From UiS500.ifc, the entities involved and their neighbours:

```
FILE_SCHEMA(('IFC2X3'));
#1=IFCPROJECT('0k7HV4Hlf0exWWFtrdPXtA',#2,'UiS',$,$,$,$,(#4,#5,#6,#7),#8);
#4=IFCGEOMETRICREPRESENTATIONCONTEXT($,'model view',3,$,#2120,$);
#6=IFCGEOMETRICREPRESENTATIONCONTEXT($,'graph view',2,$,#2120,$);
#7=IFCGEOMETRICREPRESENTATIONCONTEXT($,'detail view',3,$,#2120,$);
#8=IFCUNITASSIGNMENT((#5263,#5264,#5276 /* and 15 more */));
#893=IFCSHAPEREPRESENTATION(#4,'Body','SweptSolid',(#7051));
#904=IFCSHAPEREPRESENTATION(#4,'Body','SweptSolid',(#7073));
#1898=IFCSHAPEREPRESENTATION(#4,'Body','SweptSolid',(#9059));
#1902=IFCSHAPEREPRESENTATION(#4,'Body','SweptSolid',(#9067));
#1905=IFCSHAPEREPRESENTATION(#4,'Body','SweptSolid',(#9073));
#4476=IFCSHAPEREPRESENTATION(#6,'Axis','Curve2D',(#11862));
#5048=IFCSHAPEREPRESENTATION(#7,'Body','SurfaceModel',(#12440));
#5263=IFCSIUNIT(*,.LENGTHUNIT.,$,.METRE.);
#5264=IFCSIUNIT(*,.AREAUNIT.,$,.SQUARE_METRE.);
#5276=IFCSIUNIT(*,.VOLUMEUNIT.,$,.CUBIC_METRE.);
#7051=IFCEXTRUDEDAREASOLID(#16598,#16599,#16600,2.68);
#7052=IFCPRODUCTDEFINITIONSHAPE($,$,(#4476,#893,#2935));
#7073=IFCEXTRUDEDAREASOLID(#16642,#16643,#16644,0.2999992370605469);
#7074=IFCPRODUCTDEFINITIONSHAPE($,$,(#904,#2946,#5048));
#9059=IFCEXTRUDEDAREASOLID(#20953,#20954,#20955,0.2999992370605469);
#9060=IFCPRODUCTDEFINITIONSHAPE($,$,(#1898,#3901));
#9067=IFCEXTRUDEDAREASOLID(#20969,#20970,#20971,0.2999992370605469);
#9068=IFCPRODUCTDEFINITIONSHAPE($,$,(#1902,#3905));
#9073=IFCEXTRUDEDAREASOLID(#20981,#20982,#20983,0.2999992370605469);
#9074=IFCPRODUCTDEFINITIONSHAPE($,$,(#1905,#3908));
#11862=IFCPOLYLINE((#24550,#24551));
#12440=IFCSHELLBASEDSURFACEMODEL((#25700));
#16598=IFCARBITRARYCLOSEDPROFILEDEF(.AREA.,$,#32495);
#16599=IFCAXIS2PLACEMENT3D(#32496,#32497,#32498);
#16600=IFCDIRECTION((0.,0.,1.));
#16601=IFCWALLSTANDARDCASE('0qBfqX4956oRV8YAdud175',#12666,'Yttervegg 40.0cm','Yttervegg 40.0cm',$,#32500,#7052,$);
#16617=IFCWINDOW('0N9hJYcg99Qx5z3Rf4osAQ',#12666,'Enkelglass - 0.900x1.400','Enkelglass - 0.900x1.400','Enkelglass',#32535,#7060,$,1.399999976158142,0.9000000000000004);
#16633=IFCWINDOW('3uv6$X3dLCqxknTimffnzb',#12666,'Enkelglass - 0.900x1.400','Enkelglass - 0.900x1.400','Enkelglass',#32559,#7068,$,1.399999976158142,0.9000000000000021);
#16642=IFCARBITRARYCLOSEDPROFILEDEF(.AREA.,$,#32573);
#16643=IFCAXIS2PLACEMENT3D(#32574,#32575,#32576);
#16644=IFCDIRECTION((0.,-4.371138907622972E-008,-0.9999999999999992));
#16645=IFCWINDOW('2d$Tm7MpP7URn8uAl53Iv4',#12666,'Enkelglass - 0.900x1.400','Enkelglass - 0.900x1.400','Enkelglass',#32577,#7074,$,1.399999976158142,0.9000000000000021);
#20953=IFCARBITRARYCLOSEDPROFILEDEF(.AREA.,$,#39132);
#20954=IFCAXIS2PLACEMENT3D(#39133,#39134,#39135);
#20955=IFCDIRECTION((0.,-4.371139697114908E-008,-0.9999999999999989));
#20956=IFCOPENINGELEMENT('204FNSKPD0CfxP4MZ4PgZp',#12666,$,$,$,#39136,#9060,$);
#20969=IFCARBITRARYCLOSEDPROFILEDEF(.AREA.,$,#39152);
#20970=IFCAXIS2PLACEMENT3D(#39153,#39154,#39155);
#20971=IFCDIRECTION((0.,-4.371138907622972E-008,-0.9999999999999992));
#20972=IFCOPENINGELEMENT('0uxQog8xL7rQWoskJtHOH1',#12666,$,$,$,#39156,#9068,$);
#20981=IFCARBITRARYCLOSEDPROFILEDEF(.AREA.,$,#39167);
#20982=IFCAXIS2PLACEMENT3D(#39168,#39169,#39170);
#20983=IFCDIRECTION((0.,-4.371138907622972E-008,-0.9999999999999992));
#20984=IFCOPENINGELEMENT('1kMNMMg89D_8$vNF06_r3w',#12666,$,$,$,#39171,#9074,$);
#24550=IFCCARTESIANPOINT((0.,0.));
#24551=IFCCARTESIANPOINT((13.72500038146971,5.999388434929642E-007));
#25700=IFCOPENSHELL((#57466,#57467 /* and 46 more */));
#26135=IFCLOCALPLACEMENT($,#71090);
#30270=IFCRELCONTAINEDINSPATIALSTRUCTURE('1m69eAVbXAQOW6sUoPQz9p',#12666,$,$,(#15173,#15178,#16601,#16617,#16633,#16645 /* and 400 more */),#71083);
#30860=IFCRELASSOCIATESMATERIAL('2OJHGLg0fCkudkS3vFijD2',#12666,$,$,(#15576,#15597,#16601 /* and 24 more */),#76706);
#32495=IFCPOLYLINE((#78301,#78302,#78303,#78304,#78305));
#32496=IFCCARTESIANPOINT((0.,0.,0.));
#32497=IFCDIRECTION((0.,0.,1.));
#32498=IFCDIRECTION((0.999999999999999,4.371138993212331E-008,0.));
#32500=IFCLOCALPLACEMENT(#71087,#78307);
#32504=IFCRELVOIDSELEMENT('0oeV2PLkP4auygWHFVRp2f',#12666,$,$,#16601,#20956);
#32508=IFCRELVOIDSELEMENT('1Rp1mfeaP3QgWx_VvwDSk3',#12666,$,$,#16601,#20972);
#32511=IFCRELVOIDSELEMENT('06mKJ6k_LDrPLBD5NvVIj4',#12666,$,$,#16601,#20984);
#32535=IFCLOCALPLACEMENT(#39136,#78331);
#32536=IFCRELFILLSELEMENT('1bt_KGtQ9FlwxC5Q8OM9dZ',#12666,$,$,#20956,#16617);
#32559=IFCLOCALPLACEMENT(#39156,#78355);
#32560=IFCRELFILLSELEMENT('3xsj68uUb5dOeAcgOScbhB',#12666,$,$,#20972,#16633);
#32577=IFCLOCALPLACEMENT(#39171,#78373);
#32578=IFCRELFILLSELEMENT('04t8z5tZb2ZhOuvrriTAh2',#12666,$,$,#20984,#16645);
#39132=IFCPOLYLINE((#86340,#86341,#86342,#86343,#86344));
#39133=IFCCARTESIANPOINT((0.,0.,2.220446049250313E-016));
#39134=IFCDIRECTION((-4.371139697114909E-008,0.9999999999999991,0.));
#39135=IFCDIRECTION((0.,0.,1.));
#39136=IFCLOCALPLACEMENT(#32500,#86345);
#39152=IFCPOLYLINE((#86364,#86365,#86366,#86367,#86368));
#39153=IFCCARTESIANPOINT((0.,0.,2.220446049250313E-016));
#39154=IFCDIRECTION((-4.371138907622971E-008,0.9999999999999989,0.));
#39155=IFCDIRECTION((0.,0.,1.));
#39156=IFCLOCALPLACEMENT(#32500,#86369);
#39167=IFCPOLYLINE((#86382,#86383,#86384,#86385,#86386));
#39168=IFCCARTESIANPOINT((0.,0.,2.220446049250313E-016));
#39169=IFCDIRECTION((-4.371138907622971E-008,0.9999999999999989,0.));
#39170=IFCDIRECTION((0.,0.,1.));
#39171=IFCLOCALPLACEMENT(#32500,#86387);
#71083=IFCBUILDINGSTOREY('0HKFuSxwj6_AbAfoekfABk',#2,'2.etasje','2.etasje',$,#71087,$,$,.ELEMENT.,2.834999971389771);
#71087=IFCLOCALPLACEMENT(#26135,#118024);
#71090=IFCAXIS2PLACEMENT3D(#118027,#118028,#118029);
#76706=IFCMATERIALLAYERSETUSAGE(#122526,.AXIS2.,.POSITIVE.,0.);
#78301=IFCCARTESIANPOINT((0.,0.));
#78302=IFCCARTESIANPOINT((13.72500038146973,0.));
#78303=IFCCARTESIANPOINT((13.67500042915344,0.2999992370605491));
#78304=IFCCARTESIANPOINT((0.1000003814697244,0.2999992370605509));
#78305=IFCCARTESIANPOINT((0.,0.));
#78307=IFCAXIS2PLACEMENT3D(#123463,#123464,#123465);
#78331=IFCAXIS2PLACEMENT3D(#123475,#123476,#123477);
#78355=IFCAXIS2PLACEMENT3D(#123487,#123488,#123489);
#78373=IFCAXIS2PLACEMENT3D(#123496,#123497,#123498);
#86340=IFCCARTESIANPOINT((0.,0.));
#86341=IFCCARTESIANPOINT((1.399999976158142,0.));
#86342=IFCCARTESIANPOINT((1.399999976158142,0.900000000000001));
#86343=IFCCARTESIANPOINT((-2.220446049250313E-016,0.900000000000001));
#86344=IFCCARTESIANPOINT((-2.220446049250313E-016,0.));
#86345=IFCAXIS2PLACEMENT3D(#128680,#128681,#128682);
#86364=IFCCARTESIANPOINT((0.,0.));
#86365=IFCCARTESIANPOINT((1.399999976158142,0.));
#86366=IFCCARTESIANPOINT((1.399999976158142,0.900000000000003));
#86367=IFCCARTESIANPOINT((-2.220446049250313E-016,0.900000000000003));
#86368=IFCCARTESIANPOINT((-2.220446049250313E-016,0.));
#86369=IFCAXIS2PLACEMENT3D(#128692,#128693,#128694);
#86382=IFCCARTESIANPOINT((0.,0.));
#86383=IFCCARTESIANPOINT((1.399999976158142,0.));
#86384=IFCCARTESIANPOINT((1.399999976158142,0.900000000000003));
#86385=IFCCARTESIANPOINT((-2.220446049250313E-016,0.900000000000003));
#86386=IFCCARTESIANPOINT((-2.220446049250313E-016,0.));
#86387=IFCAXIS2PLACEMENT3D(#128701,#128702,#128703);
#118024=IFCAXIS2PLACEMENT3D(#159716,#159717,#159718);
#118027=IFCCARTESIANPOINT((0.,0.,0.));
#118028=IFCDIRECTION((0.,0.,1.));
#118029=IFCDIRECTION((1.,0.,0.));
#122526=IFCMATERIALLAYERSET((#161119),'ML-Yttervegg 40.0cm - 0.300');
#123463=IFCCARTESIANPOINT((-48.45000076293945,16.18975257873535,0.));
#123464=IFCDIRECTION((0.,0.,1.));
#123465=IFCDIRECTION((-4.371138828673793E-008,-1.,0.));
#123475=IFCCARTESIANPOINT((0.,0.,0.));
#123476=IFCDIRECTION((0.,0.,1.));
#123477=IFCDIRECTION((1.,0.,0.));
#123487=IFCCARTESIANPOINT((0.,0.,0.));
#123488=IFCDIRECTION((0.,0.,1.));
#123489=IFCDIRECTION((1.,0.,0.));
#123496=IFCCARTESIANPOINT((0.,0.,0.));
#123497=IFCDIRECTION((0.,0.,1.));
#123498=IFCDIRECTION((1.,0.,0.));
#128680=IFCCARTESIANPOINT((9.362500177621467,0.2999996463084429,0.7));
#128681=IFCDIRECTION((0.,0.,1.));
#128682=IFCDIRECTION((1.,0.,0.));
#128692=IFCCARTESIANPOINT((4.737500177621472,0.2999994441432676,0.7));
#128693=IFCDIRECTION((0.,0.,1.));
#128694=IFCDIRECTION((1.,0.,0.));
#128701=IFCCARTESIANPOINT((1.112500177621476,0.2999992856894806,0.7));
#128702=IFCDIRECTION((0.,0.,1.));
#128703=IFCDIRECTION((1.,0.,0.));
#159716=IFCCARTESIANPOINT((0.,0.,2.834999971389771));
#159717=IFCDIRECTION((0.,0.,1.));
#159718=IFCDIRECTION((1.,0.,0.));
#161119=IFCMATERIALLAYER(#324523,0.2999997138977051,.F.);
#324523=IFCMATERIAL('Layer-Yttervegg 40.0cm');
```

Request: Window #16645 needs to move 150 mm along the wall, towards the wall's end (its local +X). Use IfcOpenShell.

```python
import ifcopenshell
import ifcopenshell.api.geometry
import ifcopenshell.util.placement
import ifcopenshell.util.unit

model = ifcopenshell.open("UiS500.ifc")
unit_scale = ifcopenshell.util.unit.calculate_unit_scale(model)

window = model.by_guid("2d$Tm7MpP7URn8uAl53Iv4")
opening = window.FillsVoids[0].RelatingOpeningElement
wall = opening.VoidsElements[0].RelatingBuildingElement

wall_matrix = ifcopenshell.util.placement.get_local_placement(wall.ObjectPlacement)
shift = wall_matrix[:3, 0] * 0.15 / unit_scale
before = ifcopenshell.util.placement.get_local_placement(window.ObjectPlacement)[:3, 3].copy()

# The window is placed relative to its opening, so it follows when the opening moves.
matrix = ifcopenshell.util.placement.get_local_placement(opening.ObjectPlacement)
matrix[:3, 3] += shift
ifcopenshell.api.geometry.edit_object_placement(
    model, product=opening, matrix=matrix, is_si=False, should_transform_children=True
)

after = ifcopenshell.util.placement.get_local_placement(window.ObjectPlacement)[:3, 3]
print("window moved by", (after - before).round(3) + 0.0)

model.write("UiS500_rev.ifc")
```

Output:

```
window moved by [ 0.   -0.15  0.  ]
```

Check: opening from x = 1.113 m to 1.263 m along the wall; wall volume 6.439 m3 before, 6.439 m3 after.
